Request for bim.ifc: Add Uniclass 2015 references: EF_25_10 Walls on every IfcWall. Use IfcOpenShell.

First a look at what the model holds.

```python
import ifcopenshell

model = ifcopenshell.open("bim.ifc")
print(model.schema)
print("classifications:", [c.Name for c in model.by_type("IfcClassification")])
for ifc_class in ("IfcDoor", "IfcRoof", "IfcStair", "IfcWall", "IfcWindow"):
    print(ifc_class, len(model.by_type(ifc_class)))
```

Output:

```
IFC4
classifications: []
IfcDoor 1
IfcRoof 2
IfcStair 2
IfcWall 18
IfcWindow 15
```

```python
import ifcopenshell
import ifcopenshell.api.classification

model = ifcopenshell.open("bim.ifc")

system = ifcopenshell.api.classification.add_classification(model, classification="Uniclass 2015")

codes = {
    "IfcWall": ("EF_25_10", "Walls"),
}
for ifc_class, (code, name) in codes.items():
    products = model.by_type(ifc_class)
    ifcopenshell.api.classification.add_reference(
        model, products=products, classification=system, identification=code, name=name
    )
    print(code, len(products))

model.write("bim_rev.ifc")
```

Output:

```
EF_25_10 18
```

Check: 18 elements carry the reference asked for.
